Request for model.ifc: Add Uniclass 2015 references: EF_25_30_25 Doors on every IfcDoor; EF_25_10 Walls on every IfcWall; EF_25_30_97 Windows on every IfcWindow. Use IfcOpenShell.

First a look at what the model holds.

```python
import ifcopenshell

model = ifcopenshell.open("model.ifc")
print(model.schema)
print("classifications:", [c.Name for c in model.by_type("IfcClassification")])
for ifc_class in ("IfcDoor", "IfcRoof", "IfcStair", "IfcWall", "IfcWindow"):
    print(ifc_class, len(model.by_type(ifc_class)))
```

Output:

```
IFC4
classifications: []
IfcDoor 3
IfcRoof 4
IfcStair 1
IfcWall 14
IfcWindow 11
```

```python
import ifcopenshell
import ifcopenshell.api.classification

model = ifcopenshell.open("model.ifc")

system = ifcopenshell.api.classification.add_classification(model, classification="Uniclass 2015")

codes = {
    "IfcDoor": ("EF_25_30_25", "Doors"),
    "IfcWall": ("EF_25_10", "Walls"),
    "IfcWindow": ("EF_25_30_97", "Windows"),
}
for ifc_class, (code, name) in codes.items():
    products = model.by_type(ifc_class)
    ifcopenshell.api.classification.add_reference(
        model, products=products, classification=system, identification=code, name=name
    )
    print(code, len(products))

model.write("model_v2.ifc")
```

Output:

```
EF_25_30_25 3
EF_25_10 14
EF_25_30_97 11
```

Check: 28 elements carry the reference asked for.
